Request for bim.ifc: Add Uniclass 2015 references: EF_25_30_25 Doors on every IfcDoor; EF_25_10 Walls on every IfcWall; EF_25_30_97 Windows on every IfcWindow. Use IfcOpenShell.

First a look at what the model holds.

```python
import ifcopenshell

model = ifcopenshell.open("bim.ifc")
print(model.schema)
print("classifications:", [c.Name for c in model.by_type("IfcClassification")])
for ifc_class in ("IfcDoor", "IfcRoof", "IfcStair", "IfcWall", "IfcWindow"):
    print(ifc_class, len(model.by_type(ifc_class)))
```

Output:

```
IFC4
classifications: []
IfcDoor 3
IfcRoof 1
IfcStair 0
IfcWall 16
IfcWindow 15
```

```python
import ifcopenshell
import ifcopenshell.api.classification

model = ifcopenshell.open("bim.ifc")

system = ifcopenshell.api.classification.add_classification(model, classification="Uniclass 2015")

codes = {
    "IfcDoor": ("EF_25_30_25", "Doors"),
    "IfcWall": ("EF_25_10", "Walls"),
    "IfcWindow": ("EF_25_30_97", "Windows"),
}
for ifc_class, (code, name) in codes.items():
    products = model.by_type(ifc_class)
    ifcopenshell.api.classification.add_reference(
        model, products=products, classification=system, identification=code, name=name
    )
    print(code, len(products))

model.write("bim-out.ifc")
```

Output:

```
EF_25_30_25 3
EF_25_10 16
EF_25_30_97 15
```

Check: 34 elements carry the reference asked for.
